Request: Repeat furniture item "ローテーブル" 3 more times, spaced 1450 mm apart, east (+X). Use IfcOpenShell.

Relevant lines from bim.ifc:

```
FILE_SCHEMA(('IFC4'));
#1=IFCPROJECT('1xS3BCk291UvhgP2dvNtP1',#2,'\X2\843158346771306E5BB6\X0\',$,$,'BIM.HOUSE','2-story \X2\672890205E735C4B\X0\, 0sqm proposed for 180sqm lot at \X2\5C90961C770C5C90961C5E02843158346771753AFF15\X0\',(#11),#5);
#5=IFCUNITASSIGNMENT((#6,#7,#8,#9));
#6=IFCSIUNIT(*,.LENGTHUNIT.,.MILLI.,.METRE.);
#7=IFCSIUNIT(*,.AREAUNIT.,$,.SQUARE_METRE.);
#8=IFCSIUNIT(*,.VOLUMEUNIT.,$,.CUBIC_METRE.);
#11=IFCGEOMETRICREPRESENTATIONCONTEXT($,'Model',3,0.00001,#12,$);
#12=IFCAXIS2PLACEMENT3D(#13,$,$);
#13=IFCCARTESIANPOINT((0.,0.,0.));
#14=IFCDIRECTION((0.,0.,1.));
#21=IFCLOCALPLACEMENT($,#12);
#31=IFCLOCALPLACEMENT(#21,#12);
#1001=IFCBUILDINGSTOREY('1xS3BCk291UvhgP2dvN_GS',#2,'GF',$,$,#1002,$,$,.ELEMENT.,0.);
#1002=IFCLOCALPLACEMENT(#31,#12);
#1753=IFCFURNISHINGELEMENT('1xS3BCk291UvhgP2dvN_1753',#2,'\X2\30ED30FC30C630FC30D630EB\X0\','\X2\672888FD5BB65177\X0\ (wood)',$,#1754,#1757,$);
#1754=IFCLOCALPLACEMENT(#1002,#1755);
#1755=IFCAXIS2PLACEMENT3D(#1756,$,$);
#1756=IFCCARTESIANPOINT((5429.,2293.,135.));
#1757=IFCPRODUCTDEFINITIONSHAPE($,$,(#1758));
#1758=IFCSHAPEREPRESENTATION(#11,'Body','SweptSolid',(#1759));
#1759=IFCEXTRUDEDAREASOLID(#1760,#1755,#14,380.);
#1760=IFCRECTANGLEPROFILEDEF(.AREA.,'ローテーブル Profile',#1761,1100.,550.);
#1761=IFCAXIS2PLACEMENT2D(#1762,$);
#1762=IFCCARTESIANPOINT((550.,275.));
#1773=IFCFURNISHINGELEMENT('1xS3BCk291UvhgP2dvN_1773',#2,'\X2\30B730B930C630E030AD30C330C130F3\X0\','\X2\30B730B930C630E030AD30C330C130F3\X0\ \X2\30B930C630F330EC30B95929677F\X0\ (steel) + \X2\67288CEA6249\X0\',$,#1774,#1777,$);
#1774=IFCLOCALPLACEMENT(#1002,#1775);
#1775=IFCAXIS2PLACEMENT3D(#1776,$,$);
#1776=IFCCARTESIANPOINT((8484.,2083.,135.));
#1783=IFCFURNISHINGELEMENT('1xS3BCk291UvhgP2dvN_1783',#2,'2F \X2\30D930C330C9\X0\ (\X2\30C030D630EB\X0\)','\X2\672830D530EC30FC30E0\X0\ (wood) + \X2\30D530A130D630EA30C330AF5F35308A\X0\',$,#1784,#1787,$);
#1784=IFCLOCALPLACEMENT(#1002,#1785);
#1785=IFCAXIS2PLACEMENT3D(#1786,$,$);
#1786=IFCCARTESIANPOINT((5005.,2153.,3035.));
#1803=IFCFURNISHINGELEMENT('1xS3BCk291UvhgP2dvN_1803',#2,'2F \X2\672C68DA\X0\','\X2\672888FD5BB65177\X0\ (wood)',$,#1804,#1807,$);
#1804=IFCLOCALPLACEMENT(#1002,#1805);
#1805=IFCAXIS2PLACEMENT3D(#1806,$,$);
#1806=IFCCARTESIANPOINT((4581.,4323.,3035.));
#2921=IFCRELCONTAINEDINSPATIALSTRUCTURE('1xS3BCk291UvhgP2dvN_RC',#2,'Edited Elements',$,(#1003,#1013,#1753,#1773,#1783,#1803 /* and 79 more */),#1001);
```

```python
import numpy as np
import ifcopenshell
import ifcopenshell.api.geometry
import ifcopenshell.api.root
import ifcopenshell.util.element
import ifcopenshell.util.placement

model = ifcopenshell.open("bim.ifc")


def reuse_history(source, copy):
    """copy_class also copies each property set's owner history, people and application; keep the originals."""
    for rel in copy.IsDefinedBy:
        if rel.is_a("IfcRelDefinesByProperties") and (history := rel.RelatingPropertyDefinition.OwnerHistory):
            rel.RelatingPropertyDefinition.OwnerHistory = source.OwnerHistory
            ifcopenshell.util.element.remove_deep2(model, history)


source = model.by_guid("1xS3BCk291UvhgP2dvN_1753")
base = ifcopenshell.util.placement.get_local_placement(source.ObjectPlacement)
step = np.array([1.0, 0.0, 0.0]) * 1450.0

for i in range(1, 4):
    copy = ifcopenshell.api.root.copy_class(model, product=source)
    copy.Representation = ifcopenshell.util.element.copy_deep(
        model, source.Representation, exclude=["IfcGeometricRepresentationContext", "IfcRepresentationMap"]
    )
    reuse_history(source, copy)
    matrix = base.copy()
    matrix[:3, 3] += i * step
    print("added at", matrix[:3, 3].round(3) + 0.0)
    ifcopenshell.api.geometry.edit_object_placement(model, product=copy, matrix=matrix, is_si=False)

model.write("bim-out.ifc")
```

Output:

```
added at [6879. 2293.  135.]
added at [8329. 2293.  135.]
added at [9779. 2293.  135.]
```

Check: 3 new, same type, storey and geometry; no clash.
